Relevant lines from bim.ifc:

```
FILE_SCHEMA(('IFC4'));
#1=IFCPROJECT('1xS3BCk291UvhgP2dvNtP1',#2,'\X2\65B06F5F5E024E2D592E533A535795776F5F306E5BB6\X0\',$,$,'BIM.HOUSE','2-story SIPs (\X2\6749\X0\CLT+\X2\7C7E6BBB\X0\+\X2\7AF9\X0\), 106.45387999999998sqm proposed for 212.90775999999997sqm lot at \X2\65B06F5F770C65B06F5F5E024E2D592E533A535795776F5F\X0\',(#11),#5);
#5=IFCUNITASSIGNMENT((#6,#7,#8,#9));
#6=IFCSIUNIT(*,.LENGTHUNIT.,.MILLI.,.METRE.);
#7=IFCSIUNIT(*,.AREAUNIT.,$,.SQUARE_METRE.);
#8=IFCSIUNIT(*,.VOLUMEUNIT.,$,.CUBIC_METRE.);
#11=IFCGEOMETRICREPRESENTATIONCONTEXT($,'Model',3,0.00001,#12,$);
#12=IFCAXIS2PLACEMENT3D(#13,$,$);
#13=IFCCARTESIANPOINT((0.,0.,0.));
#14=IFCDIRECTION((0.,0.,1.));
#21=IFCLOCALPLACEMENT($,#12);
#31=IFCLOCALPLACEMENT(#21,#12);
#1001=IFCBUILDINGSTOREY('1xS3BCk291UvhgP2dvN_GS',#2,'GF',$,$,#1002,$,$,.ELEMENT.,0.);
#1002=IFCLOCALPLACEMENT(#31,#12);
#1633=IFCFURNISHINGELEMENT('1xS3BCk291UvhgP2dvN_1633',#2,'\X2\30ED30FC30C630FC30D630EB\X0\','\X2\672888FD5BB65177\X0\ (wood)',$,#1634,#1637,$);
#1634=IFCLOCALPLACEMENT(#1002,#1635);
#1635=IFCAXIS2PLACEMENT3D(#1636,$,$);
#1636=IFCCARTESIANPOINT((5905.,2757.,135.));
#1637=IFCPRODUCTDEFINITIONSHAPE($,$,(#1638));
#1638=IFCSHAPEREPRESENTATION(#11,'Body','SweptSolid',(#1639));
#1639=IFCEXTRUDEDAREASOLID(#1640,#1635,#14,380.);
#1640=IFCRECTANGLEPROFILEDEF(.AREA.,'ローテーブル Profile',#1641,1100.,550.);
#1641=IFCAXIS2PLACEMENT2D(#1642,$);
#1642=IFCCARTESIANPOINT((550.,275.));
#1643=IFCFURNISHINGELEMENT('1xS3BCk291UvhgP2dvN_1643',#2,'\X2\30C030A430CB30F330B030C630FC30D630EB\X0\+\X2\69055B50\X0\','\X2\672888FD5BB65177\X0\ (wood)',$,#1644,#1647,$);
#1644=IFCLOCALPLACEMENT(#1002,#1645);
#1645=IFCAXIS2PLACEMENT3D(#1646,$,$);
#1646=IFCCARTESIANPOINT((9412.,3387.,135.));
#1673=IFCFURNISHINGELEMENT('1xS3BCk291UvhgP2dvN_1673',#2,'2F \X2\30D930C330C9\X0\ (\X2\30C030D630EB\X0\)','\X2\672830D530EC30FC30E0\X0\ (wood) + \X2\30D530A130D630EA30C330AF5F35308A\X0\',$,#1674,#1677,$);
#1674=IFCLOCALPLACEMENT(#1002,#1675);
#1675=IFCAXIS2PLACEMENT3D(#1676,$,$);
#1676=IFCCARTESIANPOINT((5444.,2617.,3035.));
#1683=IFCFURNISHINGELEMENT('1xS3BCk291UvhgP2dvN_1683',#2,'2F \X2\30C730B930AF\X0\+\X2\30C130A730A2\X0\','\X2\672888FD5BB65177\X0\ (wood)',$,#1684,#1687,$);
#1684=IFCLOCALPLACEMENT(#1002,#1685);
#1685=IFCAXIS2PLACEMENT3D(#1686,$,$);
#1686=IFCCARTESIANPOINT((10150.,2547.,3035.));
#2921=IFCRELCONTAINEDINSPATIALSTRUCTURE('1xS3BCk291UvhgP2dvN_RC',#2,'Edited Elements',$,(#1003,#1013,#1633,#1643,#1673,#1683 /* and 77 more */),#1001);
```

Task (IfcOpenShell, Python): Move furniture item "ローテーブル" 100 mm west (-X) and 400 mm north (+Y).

```python
import ifcopenshell
import ifcopenshell.api.geometry
import ifcopenshell.util.placement
import ifcopenshell.util.unit

model = ifcopenshell.open("bim.ifc")
unit_scale = ifcopenshell.util.unit.calculate_unit_scale(model)

item = model.by_guid("1xS3BCk291UvhgP2dvN_1633")
matrix = ifcopenshell.util.placement.get_local_placement(item.ObjectPlacement)
matrix[0, 3] -= 0.1 / unit_scale
matrix[1, 3] += 0.4 / unit_scale
ifcopenshell.api.geometry.edit_object_placement(model, product=item, matrix=matrix, is_si=False)

print(ifcopenshell.util.placement.get_local_placement(item.ObjectPlacement).round(3) + 0.0)

model.write("bim_rev.ifc")
```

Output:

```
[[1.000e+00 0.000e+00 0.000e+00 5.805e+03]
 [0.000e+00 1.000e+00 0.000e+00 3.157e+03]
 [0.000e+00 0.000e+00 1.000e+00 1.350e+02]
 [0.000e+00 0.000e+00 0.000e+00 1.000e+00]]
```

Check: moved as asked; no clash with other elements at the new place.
